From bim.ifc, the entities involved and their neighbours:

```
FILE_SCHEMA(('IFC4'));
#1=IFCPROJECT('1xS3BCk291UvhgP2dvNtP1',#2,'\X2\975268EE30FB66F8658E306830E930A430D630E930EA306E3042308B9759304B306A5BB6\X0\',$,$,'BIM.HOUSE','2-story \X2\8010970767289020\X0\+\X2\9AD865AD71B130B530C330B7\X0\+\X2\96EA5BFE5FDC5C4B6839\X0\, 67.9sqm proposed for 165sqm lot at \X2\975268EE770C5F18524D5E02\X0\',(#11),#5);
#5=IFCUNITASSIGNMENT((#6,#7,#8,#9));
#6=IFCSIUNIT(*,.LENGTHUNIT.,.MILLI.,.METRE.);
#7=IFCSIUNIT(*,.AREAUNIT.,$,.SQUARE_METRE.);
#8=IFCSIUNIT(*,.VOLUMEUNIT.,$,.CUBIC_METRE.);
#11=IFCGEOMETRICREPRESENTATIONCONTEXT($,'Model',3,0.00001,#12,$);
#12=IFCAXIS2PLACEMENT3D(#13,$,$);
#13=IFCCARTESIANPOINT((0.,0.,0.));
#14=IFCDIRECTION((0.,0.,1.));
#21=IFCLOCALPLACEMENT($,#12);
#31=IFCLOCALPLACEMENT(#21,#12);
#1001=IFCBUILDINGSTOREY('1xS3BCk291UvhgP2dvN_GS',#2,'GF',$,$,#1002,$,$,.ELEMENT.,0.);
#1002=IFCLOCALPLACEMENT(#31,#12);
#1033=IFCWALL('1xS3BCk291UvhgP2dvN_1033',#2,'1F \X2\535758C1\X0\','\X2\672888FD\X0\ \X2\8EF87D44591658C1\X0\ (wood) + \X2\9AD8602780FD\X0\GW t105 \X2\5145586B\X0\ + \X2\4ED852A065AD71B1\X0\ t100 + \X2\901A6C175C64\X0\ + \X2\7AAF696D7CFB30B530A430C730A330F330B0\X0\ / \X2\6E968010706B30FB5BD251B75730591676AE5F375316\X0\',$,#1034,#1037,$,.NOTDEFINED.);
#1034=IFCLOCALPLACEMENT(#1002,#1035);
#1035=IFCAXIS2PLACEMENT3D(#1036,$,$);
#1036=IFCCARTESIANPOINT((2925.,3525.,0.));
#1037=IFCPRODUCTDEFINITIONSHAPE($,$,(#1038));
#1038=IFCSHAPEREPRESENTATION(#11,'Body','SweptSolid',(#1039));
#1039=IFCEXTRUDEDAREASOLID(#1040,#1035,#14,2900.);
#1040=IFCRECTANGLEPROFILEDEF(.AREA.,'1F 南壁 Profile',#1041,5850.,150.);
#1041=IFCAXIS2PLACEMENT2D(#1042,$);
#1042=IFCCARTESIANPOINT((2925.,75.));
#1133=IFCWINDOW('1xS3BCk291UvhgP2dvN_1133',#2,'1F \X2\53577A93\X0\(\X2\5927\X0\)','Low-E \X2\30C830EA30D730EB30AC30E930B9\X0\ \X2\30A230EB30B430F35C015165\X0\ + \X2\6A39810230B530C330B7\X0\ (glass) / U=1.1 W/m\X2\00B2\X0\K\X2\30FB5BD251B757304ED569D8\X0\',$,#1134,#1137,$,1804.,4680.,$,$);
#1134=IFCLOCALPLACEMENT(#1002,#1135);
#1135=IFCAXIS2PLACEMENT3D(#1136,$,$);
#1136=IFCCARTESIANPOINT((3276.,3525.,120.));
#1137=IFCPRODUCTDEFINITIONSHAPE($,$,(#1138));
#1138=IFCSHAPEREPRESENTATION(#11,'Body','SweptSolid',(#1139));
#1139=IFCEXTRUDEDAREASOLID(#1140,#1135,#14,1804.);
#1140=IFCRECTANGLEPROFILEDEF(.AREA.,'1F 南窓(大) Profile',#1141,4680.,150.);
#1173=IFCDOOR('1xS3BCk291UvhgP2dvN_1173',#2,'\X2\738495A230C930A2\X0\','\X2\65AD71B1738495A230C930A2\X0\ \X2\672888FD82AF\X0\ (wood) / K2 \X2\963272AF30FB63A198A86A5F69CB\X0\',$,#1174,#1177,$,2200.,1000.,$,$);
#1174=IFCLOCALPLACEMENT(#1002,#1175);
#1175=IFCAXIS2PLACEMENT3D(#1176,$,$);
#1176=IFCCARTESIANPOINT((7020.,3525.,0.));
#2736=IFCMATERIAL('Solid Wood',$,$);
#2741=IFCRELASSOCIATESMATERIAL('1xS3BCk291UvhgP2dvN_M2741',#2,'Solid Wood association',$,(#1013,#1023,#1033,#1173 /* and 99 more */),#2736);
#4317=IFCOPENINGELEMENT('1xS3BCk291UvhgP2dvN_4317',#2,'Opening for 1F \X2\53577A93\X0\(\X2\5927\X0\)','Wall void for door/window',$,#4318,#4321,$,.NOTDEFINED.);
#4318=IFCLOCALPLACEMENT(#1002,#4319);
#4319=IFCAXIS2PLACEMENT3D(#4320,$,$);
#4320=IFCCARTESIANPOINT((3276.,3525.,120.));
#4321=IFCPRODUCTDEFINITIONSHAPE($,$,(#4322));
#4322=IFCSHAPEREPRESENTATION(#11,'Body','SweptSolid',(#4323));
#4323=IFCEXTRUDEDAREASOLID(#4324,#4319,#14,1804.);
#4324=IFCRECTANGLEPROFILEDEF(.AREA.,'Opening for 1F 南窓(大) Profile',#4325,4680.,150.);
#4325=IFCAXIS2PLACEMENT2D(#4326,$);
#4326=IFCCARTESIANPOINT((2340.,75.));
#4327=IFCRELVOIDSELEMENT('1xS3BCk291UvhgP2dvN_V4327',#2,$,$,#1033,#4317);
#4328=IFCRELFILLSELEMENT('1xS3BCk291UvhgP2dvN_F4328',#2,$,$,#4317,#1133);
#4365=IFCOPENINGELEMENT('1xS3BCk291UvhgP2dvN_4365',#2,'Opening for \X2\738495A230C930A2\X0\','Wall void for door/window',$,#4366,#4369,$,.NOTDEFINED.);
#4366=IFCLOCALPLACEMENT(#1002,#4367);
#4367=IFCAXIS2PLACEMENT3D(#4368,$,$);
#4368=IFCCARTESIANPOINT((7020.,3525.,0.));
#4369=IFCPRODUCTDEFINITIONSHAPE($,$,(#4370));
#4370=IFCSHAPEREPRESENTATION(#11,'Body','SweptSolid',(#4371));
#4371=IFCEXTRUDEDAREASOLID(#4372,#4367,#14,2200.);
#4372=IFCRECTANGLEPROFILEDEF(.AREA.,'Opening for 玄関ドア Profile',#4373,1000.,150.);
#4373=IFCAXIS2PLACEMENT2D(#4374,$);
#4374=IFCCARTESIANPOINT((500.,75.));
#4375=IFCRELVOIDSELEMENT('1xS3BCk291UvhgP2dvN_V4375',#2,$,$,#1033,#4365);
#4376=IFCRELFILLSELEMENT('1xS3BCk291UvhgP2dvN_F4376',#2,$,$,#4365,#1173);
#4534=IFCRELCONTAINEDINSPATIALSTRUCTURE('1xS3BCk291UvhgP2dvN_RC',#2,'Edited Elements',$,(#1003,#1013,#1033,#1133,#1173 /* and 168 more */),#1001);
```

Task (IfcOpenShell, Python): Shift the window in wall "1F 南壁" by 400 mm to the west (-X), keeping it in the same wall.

```python
import ifcopenshell
import ifcopenshell.api.geometry
import ifcopenshell.util.placement
import ifcopenshell.util.unit

model = ifcopenshell.open("bim.ifc")
unit_scale = ifcopenshell.util.unit.calculate_unit_scale(model)

window = model.by_guid("1xS3BCk291UvhgP2dvN_1133")
opening = window.FillsVoids[0].RelatingOpeningElement
wall = opening.VoidsElements[0].RelatingBuildingElement

wall_matrix = ifcopenshell.util.placement.get_local_placement(wall.ObjectPlacement)
shift = wall_matrix[:3, 0] * -0.4 / unit_scale
before = ifcopenshell.util.placement.get_local_placement(window.ObjectPlacement)[:3, 3].copy()

# The window is not placed relative to its opening, so move both.
for product in (opening, window):
    matrix = ifcopenshell.util.placement.get_local_placement(product.ObjectPlacement)
    matrix[:3, 3] += shift
    ifcopenshell.api.geometry.edit_object_placement(model, product=product, matrix=matrix, is_si=False)

after = ifcopenshell.util.placement.get_local_placement(window.ObjectPlacement)[:3, 3]
print("window moved by", (after - before).round(3) + 0.0)

model.write("bim_edited.ifc")
```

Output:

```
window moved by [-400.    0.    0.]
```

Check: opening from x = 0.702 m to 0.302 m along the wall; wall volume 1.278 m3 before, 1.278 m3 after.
